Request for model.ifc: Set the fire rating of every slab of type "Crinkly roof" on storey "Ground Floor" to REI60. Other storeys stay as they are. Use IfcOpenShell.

First a look at what the model holds.

```python
import ifcopenshell
import ifcopenshell.util.element

model = ifcopenshell.open("model.ifc")
print(model.schema)
storey = next(s for s in model.by_type("IfcBuildingStorey") if s.Name == "Ground Floor")
slabs = [e for e in ifcopenshell.util.element.get_decomposition(storey) if e.is_a("IfcSlab")]
seen = {}
for e in slabs:
    element_type = ifcopenshell.util.element.get_type(e)
    key = (element_type.Name if element_type != e and element_type else None, ifcopenshell.util.element.get_pset(e, "Pset_SlabCommon", "FireRating"))
    seen[key] = seen.get(key, 0) + 1
for (name, value), count in sorted(seen.items(), key=str):
    print(count, "x", name, "|", value)
```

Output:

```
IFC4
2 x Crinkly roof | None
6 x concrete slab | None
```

```python
import ifcopenshell
import ifcopenshell.api.pset
import ifcopenshell.util.element

model = ifcopenshell.open("model.ifc")

storey = next(s for s in model.by_type("IfcBuildingStorey") if s.Name == "Ground Floor")
slabs = [e for e in ifcopenshell.util.element.get_decomposition(storey) if e.is_a("IfcSlab")]

count = 0
for e in slabs:
    element_type = ifcopenshell.util.element.get_type(e)
    if element_type in (None, e) or element_type.Name != "Crinkly roof":
        continue
    # add_pset returns the element's existing set when there is one.
    pset = ifcopenshell.api.pset.add_pset(model, product=e, name="Pset_SlabCommon")
    ifcopenshell.api.pset.edit_pset(model, pset=pset, properties={"FireRating": "REI60"})
    count += 1

print(count, "slabs updated")

model.write("model-out.ifc")
```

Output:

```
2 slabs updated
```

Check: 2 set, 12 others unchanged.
